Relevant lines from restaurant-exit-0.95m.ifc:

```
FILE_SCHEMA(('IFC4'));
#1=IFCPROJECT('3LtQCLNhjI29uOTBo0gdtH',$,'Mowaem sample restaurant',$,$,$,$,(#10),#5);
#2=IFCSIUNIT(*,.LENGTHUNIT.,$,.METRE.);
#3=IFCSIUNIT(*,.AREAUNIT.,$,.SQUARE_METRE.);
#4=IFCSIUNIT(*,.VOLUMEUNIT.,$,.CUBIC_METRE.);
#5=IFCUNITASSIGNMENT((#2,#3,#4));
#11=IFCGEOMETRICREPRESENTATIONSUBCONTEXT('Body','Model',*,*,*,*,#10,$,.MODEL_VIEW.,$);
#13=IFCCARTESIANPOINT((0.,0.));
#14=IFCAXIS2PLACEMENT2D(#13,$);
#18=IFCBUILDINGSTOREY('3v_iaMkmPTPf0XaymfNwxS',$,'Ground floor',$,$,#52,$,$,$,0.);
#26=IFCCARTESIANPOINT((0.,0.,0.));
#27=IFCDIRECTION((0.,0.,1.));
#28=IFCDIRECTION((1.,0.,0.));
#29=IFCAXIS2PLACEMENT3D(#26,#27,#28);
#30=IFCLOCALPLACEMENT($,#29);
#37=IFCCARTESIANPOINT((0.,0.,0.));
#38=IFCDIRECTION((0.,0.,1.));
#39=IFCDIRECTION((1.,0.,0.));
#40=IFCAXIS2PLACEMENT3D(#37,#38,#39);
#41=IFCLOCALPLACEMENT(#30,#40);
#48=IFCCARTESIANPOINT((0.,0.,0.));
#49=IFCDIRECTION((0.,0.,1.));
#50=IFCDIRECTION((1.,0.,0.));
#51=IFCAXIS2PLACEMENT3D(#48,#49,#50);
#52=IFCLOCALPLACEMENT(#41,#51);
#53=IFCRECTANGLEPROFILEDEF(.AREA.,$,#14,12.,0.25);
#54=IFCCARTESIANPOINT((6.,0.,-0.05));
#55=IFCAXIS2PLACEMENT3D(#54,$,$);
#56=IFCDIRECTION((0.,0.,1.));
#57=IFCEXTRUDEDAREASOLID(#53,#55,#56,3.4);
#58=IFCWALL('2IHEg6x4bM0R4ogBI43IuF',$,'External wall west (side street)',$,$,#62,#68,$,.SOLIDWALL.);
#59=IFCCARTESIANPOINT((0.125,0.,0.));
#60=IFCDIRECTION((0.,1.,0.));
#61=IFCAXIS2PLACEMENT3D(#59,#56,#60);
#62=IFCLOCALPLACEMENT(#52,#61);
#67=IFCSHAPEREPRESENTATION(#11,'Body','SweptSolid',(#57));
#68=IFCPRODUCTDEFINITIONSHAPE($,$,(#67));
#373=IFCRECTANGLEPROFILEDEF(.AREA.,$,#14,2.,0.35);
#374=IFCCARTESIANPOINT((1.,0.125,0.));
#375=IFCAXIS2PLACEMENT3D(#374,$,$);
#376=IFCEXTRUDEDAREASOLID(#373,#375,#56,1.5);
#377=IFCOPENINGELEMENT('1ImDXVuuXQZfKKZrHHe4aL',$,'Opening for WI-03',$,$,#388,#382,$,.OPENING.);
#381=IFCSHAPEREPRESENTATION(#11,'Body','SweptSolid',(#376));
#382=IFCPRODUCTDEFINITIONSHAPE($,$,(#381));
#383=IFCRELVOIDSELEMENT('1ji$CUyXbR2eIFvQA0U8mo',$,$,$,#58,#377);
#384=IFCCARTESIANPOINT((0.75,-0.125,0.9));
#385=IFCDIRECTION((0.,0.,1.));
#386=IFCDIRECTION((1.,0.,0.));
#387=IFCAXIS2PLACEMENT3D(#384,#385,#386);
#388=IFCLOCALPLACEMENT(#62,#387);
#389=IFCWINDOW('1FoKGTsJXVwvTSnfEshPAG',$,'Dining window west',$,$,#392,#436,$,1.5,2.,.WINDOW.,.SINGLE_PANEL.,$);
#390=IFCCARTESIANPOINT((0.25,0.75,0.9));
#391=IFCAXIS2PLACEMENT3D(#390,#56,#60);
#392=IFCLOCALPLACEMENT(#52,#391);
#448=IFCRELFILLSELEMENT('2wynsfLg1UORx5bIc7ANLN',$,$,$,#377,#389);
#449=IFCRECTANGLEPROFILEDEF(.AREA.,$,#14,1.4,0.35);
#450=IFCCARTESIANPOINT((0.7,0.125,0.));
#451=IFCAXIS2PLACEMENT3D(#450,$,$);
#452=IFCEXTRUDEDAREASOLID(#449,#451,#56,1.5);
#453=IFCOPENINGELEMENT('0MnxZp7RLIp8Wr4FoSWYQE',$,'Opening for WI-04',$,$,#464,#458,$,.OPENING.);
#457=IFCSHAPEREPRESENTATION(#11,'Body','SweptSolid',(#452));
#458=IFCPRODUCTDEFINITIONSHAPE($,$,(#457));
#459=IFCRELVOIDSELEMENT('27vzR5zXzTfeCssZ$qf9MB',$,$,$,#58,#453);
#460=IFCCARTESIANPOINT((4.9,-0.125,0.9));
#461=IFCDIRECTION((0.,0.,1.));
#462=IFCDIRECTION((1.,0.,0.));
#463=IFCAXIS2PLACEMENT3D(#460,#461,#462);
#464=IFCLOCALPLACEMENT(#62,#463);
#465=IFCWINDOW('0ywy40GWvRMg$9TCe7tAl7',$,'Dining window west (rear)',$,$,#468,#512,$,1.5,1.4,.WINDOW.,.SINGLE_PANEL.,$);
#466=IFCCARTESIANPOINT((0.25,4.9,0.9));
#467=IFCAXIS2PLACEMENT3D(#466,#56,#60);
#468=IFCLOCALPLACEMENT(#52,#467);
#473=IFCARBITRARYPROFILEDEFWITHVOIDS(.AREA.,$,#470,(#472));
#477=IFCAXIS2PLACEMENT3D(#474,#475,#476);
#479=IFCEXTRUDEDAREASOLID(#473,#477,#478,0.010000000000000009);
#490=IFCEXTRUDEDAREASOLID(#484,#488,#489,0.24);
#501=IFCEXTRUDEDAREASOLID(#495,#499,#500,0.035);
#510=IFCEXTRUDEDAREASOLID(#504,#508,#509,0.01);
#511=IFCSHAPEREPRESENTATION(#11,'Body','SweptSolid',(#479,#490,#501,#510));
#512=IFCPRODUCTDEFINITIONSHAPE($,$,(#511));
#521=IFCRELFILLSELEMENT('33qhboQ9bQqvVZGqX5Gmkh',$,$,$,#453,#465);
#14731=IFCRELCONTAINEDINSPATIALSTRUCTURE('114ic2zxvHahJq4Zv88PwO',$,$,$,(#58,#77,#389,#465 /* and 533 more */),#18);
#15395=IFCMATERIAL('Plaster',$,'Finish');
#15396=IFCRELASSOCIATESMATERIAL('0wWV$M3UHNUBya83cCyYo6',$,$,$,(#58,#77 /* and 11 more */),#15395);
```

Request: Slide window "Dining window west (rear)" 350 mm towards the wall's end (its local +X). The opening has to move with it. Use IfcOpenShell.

```python
import ifcopenshell
import ifcopenshell.api.geometry
import ifcopenshell.util.placement

model = ifcopenshell.open("restaurant-exit-0.95m.ifc")

window = model.by_guid("0ywy40GWvRMg$9TCe7tAl7")
opening = window.FillsVoids[0].RelatingOpeningElement
wall = opening.VoidsElements[0].RelatingBuildingElement

wall_matrix = ifcopenshell.util.placement.get_local_placement(wall.ObjectPlacement)
shift = wall_matrix[:3, 0] * 0.35
before = ifcopenshell.util.placement.get_local_placement(window.ObjectPlacement)[:3, 3].copy()

# The window is not placed relative to its opening, so move both.
for product in (opening, window):
    matrix = ifcopenshell.util.placement.get_local_placement(product.ObjectPlacement)
    matrix[:3, 3] += shift
    ifcopenshell.api.geometry.edit_object_placement(model, product=product, matrix=matrix, is_si=False)

after = ifcopenshell.util.placement.get_local_placement(window.ObjectPlacement)[:3, 3]
print("window moved by", (after - before).round(3) + 0.0)

model.write("restaurant-exit-0.95m_updated.ifc")
```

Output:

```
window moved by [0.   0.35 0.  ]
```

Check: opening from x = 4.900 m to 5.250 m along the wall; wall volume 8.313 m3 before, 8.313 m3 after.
